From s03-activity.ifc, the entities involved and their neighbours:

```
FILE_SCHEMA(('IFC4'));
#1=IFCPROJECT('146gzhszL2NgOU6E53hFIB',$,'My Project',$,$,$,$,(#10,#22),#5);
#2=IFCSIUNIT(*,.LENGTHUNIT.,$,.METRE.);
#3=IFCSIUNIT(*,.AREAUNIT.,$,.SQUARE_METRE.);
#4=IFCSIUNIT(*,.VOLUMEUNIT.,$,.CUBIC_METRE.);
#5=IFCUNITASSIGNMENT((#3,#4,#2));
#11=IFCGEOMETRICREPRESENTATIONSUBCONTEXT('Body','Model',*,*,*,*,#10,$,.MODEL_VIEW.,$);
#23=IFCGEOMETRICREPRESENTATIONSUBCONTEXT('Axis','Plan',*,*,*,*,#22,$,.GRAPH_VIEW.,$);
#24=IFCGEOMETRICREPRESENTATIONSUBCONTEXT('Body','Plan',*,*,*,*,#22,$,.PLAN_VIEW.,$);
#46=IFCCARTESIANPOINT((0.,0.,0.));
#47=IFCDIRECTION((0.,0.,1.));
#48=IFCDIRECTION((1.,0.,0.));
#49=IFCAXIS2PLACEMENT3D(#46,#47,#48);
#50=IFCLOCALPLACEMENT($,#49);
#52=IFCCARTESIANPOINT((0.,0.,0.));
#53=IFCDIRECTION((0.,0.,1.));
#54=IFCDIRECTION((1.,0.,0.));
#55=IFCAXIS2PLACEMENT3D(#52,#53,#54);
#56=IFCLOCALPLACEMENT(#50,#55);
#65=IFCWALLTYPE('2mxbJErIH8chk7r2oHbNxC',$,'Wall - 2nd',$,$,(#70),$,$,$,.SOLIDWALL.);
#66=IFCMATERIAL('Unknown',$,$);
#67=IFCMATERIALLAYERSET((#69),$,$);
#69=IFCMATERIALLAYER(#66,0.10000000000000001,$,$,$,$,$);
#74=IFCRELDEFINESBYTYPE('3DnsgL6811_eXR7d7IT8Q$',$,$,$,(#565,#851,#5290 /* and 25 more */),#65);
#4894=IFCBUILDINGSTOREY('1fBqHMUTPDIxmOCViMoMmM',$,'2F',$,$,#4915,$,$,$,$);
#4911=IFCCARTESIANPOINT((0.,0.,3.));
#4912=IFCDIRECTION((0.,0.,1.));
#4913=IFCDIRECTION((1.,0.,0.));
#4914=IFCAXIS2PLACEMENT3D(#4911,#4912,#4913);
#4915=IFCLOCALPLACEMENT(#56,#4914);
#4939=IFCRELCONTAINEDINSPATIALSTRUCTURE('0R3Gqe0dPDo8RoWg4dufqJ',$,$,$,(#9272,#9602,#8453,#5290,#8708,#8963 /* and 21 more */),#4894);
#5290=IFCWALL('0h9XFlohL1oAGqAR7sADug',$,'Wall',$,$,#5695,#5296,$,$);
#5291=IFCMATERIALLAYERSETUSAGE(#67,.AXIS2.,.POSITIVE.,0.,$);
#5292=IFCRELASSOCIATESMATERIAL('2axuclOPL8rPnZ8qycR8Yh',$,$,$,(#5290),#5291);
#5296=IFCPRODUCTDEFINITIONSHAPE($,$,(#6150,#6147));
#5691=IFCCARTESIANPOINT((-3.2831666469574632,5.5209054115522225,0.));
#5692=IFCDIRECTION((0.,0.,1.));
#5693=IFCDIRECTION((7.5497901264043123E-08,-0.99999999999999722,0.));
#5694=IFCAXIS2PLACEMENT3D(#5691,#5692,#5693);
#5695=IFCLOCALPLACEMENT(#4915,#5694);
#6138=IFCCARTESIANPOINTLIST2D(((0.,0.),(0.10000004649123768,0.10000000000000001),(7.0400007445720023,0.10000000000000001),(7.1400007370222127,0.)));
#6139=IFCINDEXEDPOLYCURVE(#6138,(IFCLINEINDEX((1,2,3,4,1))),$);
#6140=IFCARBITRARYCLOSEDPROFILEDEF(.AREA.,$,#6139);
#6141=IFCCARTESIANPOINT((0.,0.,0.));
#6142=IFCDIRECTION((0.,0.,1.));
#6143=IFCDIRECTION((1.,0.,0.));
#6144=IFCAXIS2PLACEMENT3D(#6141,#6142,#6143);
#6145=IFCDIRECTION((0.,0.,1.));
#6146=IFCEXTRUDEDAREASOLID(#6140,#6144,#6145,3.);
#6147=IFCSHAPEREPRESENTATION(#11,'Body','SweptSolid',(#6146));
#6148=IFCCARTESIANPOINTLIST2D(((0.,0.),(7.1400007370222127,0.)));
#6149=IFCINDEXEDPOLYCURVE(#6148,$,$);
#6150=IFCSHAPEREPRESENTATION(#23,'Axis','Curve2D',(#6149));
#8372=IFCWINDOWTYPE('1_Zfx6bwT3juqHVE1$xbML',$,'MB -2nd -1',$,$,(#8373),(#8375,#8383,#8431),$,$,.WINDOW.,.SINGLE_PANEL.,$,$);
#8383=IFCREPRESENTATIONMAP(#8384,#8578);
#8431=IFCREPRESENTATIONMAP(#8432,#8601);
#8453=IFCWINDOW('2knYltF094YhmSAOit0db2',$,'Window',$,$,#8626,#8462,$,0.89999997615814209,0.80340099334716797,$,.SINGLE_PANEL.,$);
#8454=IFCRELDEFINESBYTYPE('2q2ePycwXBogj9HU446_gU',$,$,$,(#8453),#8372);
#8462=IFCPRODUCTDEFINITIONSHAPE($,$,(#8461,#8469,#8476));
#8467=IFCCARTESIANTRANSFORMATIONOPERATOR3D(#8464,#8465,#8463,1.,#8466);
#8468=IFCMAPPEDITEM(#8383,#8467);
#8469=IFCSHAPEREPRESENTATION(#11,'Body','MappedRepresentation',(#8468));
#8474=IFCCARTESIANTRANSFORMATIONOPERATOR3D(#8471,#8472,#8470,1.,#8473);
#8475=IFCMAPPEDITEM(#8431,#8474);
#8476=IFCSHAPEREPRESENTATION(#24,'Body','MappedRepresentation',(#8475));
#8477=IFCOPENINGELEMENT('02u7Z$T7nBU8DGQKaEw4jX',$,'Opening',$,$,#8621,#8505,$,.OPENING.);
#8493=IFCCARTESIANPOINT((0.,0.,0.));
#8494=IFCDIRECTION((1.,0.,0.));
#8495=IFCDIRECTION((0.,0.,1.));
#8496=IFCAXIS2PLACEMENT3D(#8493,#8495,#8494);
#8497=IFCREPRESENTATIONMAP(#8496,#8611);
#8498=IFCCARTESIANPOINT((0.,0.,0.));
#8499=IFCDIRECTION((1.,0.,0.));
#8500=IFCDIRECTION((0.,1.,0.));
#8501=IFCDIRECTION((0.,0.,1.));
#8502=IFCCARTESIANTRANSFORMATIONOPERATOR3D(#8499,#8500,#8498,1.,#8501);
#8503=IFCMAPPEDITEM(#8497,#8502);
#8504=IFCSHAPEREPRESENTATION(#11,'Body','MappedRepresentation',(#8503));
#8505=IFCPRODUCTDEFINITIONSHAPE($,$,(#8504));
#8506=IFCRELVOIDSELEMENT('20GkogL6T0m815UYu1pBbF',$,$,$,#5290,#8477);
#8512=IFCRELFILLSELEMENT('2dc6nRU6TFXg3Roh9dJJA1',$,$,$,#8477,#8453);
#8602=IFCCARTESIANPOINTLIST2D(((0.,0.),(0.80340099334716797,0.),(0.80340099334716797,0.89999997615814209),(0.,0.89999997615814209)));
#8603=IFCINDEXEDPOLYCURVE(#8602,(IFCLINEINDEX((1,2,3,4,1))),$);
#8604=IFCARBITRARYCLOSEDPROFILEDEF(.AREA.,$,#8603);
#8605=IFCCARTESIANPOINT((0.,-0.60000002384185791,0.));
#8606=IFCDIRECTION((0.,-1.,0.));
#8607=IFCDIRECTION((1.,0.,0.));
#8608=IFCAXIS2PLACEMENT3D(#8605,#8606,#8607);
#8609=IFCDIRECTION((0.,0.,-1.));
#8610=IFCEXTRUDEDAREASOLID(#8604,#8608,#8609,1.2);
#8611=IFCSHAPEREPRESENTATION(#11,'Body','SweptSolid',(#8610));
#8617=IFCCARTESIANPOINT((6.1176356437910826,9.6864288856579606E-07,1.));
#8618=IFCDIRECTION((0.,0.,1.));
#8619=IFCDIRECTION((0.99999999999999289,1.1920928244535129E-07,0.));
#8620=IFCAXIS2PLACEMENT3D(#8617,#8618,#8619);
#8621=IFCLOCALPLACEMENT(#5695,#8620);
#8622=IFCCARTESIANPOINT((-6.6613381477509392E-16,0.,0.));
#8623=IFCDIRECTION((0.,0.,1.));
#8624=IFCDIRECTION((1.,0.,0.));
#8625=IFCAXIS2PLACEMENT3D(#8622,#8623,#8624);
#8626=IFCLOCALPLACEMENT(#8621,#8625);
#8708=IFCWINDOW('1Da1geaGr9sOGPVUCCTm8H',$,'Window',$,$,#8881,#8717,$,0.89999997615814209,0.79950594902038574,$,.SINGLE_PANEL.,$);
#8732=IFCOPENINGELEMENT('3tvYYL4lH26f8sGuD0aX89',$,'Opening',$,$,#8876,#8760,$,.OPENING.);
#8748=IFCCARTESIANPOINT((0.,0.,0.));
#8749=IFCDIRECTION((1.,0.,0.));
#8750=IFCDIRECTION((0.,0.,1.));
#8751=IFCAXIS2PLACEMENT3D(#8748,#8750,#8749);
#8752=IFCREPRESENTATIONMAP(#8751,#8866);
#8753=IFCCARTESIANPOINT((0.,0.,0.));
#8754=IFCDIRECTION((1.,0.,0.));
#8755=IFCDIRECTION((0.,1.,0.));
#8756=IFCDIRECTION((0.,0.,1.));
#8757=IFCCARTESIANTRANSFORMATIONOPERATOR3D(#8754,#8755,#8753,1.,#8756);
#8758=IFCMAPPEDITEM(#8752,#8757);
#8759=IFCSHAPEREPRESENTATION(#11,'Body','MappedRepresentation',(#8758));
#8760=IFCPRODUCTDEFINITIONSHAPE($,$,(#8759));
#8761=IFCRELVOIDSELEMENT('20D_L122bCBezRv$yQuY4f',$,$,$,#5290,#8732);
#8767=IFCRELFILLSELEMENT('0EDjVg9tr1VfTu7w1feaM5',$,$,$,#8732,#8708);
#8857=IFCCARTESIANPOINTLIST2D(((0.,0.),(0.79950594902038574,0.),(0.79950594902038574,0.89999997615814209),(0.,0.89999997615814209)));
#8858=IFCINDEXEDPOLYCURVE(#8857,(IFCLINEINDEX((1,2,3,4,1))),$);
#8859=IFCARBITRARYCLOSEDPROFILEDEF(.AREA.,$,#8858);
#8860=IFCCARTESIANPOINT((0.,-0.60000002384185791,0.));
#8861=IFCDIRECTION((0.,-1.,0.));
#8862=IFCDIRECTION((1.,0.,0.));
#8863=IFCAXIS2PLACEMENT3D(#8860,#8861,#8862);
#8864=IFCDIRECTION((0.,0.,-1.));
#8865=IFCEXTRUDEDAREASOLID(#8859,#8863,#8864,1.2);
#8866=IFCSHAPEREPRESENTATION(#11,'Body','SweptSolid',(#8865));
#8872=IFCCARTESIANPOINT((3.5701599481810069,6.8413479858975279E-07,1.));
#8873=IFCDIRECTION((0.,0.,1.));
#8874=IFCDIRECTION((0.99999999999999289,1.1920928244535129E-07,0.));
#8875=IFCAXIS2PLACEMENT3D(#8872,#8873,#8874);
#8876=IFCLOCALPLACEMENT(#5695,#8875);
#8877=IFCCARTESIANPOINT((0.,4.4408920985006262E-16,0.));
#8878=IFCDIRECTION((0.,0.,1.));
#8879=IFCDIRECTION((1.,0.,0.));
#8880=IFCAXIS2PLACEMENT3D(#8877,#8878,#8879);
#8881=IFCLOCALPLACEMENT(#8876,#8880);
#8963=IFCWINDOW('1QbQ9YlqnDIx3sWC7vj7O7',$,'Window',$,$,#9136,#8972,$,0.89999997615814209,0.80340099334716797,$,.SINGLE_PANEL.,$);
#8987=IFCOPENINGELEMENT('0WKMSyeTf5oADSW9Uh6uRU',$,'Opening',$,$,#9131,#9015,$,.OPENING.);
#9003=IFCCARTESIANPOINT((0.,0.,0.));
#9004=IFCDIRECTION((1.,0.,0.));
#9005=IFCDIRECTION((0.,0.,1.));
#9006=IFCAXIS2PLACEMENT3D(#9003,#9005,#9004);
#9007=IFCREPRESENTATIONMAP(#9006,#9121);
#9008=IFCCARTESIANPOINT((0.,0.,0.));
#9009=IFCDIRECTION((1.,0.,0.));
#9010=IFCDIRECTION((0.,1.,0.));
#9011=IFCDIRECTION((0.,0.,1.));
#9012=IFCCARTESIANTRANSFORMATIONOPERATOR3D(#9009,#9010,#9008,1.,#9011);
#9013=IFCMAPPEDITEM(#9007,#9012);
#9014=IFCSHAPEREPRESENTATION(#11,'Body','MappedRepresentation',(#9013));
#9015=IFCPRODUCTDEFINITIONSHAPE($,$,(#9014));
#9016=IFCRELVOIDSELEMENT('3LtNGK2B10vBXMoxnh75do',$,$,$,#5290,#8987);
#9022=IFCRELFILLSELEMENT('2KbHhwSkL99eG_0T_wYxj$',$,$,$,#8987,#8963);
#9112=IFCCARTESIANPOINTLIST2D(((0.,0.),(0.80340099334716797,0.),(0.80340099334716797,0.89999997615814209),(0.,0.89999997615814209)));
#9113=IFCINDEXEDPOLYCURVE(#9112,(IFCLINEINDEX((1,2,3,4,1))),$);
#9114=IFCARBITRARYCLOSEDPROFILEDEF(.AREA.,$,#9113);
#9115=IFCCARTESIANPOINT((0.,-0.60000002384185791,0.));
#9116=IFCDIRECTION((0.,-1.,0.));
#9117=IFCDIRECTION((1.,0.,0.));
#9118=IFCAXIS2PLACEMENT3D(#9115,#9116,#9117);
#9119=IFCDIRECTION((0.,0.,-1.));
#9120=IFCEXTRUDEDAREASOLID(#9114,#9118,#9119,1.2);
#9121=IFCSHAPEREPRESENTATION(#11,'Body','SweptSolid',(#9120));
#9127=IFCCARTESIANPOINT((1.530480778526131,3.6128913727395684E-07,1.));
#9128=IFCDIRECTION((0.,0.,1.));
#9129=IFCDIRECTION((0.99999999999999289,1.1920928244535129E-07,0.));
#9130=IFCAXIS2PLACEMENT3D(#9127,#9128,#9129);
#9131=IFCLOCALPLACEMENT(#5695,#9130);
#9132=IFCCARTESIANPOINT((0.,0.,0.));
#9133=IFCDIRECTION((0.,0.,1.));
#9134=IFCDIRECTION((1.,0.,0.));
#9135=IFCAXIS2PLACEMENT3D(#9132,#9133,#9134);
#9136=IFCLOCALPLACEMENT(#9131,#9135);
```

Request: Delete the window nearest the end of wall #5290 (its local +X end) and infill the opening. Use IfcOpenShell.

```python
import ifcopenshell
import ifcopenshell.api.feature
import ifcopenshell.api.root
import ifcopenshell.geom
import ifcopenshell.util.shape

model = ifcopenshell.open("s03-activity.ifc")
settings = ifcopenshell.geom.settings()


def volume(element):
    """Net volume in cubic metres, openings subtracted."""
    shape = ifcopenshell.geom.create_shape(settings, element)
    return ifcopenshell.util.shape.get_volume(shape.geometry)


window = model.by_id(8453)
opening = window.FillsVoids[0].RelatingOpeningElement
wall = opening.VoidsElements[0].RelatingBuildingElement
before = volume(wall)

ifcopenshell.api.root.remove_product(model, product=window)
ifcopenshell.api.feature.remove_feature(model, feature=opening)

after = volume(wall)

print(f"wall volume {before:.3f} -> {after:.3f} m3")

model.write("s03-activity_edited.ifc")
```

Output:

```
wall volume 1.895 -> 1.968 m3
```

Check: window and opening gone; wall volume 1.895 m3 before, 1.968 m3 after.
